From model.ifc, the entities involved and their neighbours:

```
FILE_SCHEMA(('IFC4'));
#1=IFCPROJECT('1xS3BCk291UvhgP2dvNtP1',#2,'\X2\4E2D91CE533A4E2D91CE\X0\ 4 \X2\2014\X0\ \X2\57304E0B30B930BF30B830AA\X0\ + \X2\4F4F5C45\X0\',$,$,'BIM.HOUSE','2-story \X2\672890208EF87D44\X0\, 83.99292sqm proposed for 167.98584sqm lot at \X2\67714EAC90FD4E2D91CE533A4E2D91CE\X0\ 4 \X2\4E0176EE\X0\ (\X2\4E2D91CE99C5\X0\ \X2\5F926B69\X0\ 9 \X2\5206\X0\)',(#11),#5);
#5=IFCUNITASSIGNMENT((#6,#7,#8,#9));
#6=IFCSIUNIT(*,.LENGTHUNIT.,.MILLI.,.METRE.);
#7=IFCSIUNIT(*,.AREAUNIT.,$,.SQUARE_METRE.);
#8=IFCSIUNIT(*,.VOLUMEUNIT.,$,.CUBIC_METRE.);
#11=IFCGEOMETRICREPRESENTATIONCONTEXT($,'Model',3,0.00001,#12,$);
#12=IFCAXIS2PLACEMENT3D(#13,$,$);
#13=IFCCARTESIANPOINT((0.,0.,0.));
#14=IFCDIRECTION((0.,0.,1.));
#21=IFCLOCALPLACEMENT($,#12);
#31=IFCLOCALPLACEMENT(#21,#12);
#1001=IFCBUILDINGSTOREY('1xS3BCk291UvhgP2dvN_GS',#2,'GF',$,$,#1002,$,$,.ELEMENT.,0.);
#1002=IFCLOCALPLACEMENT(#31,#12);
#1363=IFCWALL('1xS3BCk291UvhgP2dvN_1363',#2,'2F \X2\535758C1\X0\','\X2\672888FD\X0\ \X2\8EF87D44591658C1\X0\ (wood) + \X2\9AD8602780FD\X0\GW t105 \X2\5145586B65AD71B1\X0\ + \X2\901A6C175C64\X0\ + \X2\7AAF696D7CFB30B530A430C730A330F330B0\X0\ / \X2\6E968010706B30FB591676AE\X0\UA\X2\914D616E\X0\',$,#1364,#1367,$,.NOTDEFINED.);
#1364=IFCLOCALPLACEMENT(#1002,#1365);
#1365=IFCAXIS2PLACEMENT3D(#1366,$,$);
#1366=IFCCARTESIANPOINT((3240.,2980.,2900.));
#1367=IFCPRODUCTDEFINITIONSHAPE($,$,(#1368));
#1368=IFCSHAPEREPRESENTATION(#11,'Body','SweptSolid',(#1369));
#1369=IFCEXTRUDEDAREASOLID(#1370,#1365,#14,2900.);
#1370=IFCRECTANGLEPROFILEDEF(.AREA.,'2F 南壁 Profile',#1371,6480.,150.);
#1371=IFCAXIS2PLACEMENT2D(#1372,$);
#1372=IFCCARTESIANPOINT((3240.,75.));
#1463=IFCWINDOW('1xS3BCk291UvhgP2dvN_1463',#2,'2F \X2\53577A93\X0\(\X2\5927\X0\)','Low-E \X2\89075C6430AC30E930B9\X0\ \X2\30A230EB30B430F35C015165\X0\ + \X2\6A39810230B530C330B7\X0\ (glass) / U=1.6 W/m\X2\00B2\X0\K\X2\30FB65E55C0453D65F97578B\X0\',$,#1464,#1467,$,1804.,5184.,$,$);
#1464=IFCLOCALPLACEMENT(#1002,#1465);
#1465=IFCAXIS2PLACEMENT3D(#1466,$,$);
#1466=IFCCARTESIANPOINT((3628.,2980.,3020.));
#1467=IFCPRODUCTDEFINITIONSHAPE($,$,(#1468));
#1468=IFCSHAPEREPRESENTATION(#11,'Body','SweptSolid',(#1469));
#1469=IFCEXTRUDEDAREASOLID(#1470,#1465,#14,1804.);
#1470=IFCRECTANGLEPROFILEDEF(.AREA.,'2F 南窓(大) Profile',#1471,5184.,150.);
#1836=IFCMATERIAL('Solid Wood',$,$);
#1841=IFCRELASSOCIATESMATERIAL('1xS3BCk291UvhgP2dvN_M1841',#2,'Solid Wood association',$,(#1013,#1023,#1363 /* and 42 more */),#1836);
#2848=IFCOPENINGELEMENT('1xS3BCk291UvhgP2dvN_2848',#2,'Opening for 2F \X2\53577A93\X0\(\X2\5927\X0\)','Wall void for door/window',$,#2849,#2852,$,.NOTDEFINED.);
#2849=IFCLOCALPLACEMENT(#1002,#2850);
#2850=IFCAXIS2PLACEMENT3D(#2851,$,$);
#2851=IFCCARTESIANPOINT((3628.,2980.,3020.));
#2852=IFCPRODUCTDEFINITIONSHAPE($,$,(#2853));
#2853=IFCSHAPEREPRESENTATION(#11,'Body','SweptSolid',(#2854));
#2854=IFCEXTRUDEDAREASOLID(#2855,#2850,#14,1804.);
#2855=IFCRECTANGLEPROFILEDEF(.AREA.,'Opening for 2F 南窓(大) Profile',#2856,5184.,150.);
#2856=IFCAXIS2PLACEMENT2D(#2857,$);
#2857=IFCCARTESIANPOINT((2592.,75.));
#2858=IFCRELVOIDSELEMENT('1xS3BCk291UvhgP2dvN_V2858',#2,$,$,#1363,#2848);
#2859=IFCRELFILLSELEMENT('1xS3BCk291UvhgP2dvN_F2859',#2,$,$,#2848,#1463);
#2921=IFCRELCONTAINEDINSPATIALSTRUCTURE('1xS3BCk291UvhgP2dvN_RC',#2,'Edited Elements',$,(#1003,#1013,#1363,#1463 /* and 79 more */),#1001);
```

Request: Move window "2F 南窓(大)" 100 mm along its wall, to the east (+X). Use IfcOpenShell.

```python
import ifcopenshell
import ifcopenshell.api.geometry
import ifcopenshell.util.placement

model = ifcopenshell.open("model.ifc")

window = model.by_id(1463)
opening = window.FillsVoids[0].RelatingOpeningElement
wall = opening.VoidsElements[0].RelatingBuildingElement

wall_matrix = ifcopenshell.util.placement.get_local_placement(wall.ObjectPlacement)
shift = wall_matrix[:3, 0] * 100.0
before = ifcopenshell.util.placement.get_local_placement(window.ObjectPlacement)[:3, 3].copy()

# The window is not placed relative to its opening, so move both.
for product in (opening, window):
    matrix = ifcopenshell.util.placement.get_local_placement(product.ObjectPlacement)
    matrix[:3, 3] += shift
    ifcopenshell.api.geometry.edit_object_placement(model, product=product, matrix=matrix, is_si=False)

after = ifcopenshell.util.placement.get_local_placement(window.ObjectPlacement)[:3, 3]
print("window moved by", (after - before).round(3) + 0.0)

model.write("model-out.ifc")
```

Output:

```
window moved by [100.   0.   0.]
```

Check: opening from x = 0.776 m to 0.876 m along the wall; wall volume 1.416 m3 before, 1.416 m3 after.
